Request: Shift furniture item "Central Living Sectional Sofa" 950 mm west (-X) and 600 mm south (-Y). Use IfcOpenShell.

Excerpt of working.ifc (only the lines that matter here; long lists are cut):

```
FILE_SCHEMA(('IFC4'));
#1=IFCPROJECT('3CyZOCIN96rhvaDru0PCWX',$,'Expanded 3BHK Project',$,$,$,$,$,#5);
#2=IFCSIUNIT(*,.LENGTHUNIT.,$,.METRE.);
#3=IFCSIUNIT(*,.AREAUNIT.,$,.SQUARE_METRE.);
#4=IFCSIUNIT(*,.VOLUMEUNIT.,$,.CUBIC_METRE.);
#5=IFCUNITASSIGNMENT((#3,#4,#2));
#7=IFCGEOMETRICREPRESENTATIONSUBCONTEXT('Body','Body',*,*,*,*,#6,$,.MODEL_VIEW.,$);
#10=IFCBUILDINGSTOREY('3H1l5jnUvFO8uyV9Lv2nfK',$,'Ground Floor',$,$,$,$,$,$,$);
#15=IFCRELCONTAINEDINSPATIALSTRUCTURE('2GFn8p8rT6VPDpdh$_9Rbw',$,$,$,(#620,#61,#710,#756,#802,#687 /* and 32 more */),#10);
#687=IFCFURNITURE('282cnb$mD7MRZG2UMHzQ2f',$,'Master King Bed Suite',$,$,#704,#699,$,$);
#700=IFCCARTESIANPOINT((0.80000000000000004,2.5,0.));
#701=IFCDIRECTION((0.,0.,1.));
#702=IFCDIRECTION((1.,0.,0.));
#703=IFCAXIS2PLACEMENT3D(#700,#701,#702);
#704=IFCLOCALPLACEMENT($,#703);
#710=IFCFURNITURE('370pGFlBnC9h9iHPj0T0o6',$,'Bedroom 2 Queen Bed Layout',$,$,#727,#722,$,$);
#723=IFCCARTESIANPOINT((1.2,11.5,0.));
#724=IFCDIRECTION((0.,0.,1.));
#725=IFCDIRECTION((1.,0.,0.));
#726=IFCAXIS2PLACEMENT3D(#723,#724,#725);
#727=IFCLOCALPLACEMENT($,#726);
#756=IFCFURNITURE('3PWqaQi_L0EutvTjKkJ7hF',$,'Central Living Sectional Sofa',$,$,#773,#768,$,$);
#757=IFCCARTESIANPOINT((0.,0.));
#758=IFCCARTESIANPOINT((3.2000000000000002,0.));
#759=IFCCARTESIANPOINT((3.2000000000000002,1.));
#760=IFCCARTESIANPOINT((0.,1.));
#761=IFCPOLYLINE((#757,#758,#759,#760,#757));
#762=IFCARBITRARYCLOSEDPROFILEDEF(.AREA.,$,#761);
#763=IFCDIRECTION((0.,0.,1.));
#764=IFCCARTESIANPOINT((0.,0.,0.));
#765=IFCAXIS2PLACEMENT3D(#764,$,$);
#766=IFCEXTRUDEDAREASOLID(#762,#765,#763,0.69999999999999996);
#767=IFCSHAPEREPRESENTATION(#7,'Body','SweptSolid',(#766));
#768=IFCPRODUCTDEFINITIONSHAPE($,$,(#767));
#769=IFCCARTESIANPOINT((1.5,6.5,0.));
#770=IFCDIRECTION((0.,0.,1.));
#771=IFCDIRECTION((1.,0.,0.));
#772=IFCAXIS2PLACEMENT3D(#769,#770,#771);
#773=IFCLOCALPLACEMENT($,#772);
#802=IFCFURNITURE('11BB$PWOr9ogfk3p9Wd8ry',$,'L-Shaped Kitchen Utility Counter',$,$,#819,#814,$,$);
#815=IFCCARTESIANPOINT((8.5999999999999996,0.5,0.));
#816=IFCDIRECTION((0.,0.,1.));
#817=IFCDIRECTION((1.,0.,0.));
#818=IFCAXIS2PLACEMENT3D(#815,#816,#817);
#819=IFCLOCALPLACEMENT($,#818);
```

```python
import ifcopenshell
import ifcopenshell.api.geometry
import ifcopenshell.util.placement

model = ifcopenshell.open("working.ifc")

item = model.by_guid("3PWqaQi_L0EutvTjKkJ7hF")
matrix = ifcopenshell.util.placement.get_local_placement(item.ObjectPlacement)
matrix[0, 3] -= 0.95
matrix[1, 3] -= 0.6
ifcopenshell.api.geometry.edit_object_placement(model, product=item, matrix=matrix, is_si=False)

print(ifcopenshell.util.placement.get_local_placement(item.ObjectPlacement).round(3) + 0.0)

model.write("working-out.ifc")
```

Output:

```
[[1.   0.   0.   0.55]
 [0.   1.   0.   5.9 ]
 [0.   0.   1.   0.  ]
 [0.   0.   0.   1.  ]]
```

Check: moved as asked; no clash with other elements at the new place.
